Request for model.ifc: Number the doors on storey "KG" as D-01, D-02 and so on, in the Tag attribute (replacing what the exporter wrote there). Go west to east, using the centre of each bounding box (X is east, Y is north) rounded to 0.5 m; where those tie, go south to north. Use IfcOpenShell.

First a look at what the model holds.

```python
import ifcopenshell
import ifcopenshell.util.element
import ifcopenshell.util.placement

model = ifcopenshell.open("model.ifc")
print(model.schema)
storey = next(s for s in model.by_type("IfcBuildingStorey") if s.Name == "KG")
doors = [e for e in ifcopenshell.util.element.get_decomposition(storey) if e.is_a("IfcDoor")]
for e in sorted(doors, key=lambda e: e.id()):
    origin = ifcopenshell.util.placement.get_local_placement(e.ObjectPlacement)[:3, 3]
    print(e.id(), e.Tag, e.Name, origin.round(2) + 0.0, sep=" | ")
```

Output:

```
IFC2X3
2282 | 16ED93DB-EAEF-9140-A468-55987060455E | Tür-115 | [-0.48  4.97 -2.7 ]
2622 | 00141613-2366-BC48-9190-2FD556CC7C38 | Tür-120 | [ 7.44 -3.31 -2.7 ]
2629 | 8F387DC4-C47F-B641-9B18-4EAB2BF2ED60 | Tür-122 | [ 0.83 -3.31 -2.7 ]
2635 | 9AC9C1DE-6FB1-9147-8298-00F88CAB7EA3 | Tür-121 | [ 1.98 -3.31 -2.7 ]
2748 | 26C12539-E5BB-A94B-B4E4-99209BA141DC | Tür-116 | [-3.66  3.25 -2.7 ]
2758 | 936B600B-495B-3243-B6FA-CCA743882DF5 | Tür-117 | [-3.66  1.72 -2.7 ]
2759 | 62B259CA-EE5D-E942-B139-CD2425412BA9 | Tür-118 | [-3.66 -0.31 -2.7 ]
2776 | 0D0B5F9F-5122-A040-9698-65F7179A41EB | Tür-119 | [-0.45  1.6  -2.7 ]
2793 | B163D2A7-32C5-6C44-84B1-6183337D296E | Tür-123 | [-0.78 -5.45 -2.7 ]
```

```python
import ifcopenshell
import ifcopenshell.geom
import ifcopenshell.util.element
import ifcopenshell.util.shape

model = ifcopenshell.open("model.ifc")
settings = ifcopenshell.geom.settings()
settings.set("use-world-coords", True)


def centre(element):
    shape = ifcopenshell.geom.create_shape(settings, element)
    return ifcopenshell.util.shape.get_bbox_centroid(shape.geometry)


storey = next(s for s in model.by_type("IfcBuildingStorey") if s.Name == "KG")
doors = [e for e in ifcopenshell.util.element.get_decomposition(storey) if e.is_a("IfcDoor")]

# Insertion points can sit at a corner or the storey origin, so sort by the geometry (in metres).
centres = {e: centre(e) for e in doors}
doors.sort(key=lambda e: (round(centres[e][0] / 0.5), centres[e][1]))

for i, e in enumerate(doors, start=1):
    number = f"D-{i:02d}"
    e.Tag = number
    print(e.id(), number)

model.write("model-out.ifc")
```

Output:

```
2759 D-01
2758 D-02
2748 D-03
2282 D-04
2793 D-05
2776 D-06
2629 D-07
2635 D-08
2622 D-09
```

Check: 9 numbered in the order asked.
